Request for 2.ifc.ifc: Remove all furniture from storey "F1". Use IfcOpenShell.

First a look at what the model holds.

```python
import ifcopenshell
import ifcopenshell.util.element

model = ifcopenshell.open("2.ifc.ifc")
print(model.schema)
storey = next(s for s in model.by_type("IfcBuildingStorey") if s.Name == "F1")
furniture = [e for e in ifcopenshell.util.element.get_decomposition(storey) if e.is_a("IfcFurnishingElement")]
seen = {}
for e in furniture:
    element_type = ifcopenshell.util.element.get_type(e)
    name = element_type.Name if element_type not in (None, e) else None
    seen[name] = seen.get(name, 0) + 1
for name, count in sorted(seen.items(), key=str):
    print(count, "x", name)
```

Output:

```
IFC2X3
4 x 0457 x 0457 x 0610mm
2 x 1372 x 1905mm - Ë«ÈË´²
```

```python
import ifcopenshell
import ifcopenshell.api.root
import ifcopenshell.util.element

model = ifcopenshell.open("2.ifc.ifc")

storey = next(s for s in model.by_type("IfcBuildingStorey") if s.Name == "F1")
furniture = [e for e in ifcopenshell.util.element.get_decomposition(storey) if e.is_a("IfcFurnishingElement")]

for e in furniture:
    ifcopenshell.api.root.remove_product(model, product=e)
print(len(furniture), "removed")

model.write("2.ifc-out.ifc")
```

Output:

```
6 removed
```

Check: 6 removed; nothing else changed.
